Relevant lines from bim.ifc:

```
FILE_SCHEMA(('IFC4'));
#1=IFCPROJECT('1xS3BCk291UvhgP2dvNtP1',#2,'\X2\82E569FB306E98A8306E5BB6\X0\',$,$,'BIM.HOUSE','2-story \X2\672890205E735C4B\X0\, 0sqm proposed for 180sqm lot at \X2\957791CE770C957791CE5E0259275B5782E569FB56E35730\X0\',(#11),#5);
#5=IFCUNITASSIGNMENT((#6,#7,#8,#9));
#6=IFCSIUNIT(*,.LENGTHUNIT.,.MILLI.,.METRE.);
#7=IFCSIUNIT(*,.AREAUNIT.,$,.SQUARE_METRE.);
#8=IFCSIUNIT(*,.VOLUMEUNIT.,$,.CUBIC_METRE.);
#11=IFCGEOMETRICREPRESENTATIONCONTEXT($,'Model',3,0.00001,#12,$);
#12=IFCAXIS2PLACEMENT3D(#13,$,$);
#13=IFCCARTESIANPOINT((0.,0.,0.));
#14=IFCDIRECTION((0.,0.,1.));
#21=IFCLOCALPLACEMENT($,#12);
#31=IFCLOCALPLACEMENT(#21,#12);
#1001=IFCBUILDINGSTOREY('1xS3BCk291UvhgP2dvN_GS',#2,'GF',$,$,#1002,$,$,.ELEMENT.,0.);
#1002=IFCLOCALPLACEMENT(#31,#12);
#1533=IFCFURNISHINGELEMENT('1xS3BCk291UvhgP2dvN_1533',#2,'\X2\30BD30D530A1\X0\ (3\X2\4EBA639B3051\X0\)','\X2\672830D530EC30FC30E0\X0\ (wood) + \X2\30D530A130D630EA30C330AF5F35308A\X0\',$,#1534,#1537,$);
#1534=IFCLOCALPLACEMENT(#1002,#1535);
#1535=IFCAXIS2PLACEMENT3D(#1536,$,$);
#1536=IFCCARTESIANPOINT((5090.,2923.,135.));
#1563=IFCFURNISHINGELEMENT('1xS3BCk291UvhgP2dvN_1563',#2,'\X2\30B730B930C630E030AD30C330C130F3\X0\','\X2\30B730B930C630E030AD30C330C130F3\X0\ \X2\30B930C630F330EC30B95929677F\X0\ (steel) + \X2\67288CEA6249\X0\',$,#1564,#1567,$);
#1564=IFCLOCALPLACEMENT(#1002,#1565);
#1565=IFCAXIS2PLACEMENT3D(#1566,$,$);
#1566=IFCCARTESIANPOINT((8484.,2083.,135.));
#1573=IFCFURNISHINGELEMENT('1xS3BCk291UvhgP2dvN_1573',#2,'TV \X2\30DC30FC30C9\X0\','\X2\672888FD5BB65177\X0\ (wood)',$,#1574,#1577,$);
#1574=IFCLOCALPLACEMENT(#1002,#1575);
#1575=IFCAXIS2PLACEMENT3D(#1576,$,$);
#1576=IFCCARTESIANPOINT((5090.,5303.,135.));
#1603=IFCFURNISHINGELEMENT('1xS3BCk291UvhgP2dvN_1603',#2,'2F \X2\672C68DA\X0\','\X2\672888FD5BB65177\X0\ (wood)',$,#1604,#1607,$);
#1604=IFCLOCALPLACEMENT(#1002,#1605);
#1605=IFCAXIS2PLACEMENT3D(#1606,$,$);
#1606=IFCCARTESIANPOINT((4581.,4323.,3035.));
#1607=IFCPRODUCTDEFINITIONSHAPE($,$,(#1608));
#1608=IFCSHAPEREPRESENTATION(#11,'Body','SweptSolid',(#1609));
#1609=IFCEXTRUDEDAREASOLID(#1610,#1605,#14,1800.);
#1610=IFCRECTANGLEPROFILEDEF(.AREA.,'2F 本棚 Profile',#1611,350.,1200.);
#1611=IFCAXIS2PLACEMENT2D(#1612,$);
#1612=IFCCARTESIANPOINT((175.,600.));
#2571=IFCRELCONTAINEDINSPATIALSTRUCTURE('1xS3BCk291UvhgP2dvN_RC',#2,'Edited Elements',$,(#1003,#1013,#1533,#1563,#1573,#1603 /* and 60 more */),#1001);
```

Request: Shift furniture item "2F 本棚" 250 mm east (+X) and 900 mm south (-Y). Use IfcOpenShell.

```python
import ifcopenshell
import ifcopenshell.api.geometry
import ifcopenshell.util.placement

model = ifcopenshell.open("bim.ifc")

item = model.by_guid("1xS3BCk291UvhgP2dvN_1603")
matrix = ifcopenshell.util.placement.get_local_placement(item.ObjectPlacement)
matrix[0, 3] += 250.0
matrix[1, 3] -= 900.0
ifcopenshell.api.geometry.edit_object_placement(model, product=item, matrix=matrix, is_si=False)

print(ifcopenshell.util.placement.get_local_placement(item.ObjectPlacement).round(3) + 0.0)

model.write("bim-out.ifc")
```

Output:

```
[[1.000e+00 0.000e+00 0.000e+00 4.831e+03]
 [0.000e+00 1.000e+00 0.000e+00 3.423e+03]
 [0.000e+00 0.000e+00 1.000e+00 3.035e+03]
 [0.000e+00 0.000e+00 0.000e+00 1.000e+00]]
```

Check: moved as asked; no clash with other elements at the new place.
